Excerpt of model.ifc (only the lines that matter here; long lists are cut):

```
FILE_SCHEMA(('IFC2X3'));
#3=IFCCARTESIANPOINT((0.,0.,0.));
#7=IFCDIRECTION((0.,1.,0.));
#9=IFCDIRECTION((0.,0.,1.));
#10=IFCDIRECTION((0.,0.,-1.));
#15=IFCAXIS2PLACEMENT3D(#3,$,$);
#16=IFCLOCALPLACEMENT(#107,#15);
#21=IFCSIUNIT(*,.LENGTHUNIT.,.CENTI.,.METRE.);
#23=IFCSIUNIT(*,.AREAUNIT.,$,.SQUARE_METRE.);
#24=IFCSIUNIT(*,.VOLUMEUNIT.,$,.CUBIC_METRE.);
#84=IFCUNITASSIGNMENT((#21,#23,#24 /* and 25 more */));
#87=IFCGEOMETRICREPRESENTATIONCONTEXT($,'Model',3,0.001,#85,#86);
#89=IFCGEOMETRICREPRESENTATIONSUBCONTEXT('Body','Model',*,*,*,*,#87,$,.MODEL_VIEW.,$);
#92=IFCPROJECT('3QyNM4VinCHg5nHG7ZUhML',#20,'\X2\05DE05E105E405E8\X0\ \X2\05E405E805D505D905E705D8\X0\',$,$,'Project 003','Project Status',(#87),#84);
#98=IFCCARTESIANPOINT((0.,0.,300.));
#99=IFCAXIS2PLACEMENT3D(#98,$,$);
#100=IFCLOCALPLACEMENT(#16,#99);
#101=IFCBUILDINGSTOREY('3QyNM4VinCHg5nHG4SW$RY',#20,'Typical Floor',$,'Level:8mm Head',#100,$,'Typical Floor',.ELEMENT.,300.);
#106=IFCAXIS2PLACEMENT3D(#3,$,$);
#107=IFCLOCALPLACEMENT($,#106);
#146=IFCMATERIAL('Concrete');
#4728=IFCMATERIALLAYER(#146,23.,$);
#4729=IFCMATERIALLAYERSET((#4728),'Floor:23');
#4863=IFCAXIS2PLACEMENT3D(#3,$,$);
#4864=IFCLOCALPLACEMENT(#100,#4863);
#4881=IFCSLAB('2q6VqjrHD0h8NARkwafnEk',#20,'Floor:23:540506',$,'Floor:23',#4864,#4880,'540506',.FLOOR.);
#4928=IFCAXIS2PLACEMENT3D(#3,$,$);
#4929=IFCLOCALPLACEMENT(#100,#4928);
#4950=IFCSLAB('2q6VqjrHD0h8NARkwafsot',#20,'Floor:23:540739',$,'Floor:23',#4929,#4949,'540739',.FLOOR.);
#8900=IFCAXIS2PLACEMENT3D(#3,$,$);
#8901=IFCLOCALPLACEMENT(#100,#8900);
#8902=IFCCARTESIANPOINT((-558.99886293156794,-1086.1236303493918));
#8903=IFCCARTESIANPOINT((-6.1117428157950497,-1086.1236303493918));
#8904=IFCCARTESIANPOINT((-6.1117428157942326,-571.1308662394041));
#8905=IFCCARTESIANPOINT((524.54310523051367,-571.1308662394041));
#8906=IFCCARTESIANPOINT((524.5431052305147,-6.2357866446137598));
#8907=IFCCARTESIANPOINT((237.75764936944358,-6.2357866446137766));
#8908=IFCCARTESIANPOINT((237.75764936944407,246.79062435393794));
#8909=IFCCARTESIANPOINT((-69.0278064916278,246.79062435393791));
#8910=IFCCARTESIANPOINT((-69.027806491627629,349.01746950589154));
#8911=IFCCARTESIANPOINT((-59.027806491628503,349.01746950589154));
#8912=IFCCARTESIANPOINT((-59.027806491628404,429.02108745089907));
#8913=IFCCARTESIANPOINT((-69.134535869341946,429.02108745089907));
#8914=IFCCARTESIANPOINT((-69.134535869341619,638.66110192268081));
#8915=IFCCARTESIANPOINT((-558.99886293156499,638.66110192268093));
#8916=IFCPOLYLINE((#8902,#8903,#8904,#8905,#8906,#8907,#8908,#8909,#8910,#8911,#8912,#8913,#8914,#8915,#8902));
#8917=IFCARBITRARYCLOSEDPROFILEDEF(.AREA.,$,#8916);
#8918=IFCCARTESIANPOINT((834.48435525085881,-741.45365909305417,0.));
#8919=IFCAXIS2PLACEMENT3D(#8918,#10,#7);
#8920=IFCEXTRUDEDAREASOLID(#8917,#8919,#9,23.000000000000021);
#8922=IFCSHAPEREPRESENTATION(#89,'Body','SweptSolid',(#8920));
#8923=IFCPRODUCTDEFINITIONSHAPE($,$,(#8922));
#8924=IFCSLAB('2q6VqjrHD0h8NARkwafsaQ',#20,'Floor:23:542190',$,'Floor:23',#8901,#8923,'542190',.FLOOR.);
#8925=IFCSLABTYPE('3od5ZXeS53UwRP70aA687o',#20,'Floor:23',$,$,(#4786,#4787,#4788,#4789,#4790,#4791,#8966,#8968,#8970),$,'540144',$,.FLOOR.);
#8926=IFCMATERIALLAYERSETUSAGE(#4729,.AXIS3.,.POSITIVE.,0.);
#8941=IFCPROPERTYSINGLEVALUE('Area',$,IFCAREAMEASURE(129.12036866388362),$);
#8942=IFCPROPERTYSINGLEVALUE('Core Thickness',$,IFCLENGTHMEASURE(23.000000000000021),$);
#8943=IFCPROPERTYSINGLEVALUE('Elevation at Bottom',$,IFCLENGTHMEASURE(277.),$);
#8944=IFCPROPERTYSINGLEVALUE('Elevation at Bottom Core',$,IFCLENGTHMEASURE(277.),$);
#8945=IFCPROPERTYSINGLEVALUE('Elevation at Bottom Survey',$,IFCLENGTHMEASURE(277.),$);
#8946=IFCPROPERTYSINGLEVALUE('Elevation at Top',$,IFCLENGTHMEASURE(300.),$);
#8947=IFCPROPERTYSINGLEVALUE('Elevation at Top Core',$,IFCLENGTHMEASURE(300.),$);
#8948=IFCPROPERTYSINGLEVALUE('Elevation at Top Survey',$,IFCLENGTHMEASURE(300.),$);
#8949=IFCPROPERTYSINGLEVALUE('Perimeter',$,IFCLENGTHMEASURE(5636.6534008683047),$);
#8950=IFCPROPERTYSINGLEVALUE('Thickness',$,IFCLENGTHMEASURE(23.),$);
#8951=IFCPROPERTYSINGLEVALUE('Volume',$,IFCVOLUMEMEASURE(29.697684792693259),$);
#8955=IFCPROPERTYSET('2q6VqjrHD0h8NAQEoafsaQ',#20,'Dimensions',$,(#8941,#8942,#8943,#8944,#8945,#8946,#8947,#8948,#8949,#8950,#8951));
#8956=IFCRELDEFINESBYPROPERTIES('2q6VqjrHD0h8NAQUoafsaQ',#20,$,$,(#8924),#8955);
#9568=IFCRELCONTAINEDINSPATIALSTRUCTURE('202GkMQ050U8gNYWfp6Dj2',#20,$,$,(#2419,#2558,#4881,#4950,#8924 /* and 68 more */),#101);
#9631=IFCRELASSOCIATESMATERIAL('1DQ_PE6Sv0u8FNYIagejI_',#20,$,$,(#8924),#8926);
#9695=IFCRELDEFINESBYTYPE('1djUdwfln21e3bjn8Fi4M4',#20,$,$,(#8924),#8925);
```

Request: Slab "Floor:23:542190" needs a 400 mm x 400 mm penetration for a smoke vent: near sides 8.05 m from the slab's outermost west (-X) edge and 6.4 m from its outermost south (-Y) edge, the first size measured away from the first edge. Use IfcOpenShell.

```python
import numpy as np
import ifcopenshell
import ifcopenshell.api.feature
import ifcopenshell.api.geometry
import ifcopenshell.api.pset
import ifcopenshell.api.root
import ifcopenshell.geom
import ifcopenshell.util.element
import ifcopenshell.util.placement
import ifcopenshell.util.representation
import ifcopenshell.util.shape
import ifcopenshell.util.unit

model = ifcopenshell.open("model.ifc")
unit_scale = ifcopenshell.util.unit.calculate_unit_scale(model)
area_scale = ifcopenshell.util.unit.calculate_unit_scale(model, "AREAUNIT")
volume_scale = ifcopenshell.util.unit.calculate_unit_scale(model, "VOLUMEUNIT")
settings = ifcopenshell.geom.settings()


def volume(element):
    """Net volume in cubic metres, openings subtracted."""
    shape = ifcopenshell.geom.create_shape(settings, element)
    return ifcopenshell.util.shape.get_volume(shape.geometry)


slab = model.by_guid("2q6VqjrHD0h8NARkwafsaQ")
before = volume(slab)

# Extent in the slab's own axes, in metres. The edges named are its -X and -Y sides.
slab_shape = ifcopenshell.geom.create_shape(settings, slab)
vertices = ifcopenshell.util.shape.get_vertices(slab_shape.geometry)
x_min, y_min, bottom = vertices.min(axis=0)
top = vertices[:, 2].max()

opening = ifcopenshell.api.root.create_entity(model, ifc_class="IfcOpeningElement", name="Smoke vent opening")
context = ifcopenshell.util.representation.get_context(model, "Model", "Body", "MODEL_VIEW")
width, depth = 0.4, 0.4
outline = [(0.0, 0.0), (width, 0.0), (width, depth), (0.0, depth), (0.0, 0.0)]
# Overshoot both faces by 50 mm so the cut is clean.
shape = ifcopenshell.api.geometry.add_slab_representation(
    model, context=context, depth=top - bottom + 0.1, polyline=outline
)
ifcopenshell.api.geometry.assign_representation(model, product=opening, representation=shape)

matrix = ifcopenshell.util.placement.get_local_placement(slab.ObjectPlacement)
matrix[:, 3] = matrix @ np.append(np.array([x_min + 8.05, y_min + 6.4, bottom - 0.05]) / unit_scale, 1.0)
ifcopenshell.api.geometry.edit_object_placement(model, product=opening, matrix=matrix, is_si=False)
ifcopenshell.api.feature.add_feature(model, feature=opening, element=slab)

after = volume(slab)

# Update the slab's stored quantities.
pset = model.by_id(ifcopenshell.util.element.get_pset(slab, "Dimensions", should_inherit=False)["id"])
ifcopenshell.api.pset.edit_pset(model, pset=pset, properties={
    "Area": model.create_entity("IfcAreaMeasure", after / (top - bottom) / area_scale),
    "Volume": model.create_entity("IfcVolumeMeasure", after / volume_scale),
})

print(f"slab volume {before:.3f} -> {after:.3f} m3")

model.write("model-out.ifc")
```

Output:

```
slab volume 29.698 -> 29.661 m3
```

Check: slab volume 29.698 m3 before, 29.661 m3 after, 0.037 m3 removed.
